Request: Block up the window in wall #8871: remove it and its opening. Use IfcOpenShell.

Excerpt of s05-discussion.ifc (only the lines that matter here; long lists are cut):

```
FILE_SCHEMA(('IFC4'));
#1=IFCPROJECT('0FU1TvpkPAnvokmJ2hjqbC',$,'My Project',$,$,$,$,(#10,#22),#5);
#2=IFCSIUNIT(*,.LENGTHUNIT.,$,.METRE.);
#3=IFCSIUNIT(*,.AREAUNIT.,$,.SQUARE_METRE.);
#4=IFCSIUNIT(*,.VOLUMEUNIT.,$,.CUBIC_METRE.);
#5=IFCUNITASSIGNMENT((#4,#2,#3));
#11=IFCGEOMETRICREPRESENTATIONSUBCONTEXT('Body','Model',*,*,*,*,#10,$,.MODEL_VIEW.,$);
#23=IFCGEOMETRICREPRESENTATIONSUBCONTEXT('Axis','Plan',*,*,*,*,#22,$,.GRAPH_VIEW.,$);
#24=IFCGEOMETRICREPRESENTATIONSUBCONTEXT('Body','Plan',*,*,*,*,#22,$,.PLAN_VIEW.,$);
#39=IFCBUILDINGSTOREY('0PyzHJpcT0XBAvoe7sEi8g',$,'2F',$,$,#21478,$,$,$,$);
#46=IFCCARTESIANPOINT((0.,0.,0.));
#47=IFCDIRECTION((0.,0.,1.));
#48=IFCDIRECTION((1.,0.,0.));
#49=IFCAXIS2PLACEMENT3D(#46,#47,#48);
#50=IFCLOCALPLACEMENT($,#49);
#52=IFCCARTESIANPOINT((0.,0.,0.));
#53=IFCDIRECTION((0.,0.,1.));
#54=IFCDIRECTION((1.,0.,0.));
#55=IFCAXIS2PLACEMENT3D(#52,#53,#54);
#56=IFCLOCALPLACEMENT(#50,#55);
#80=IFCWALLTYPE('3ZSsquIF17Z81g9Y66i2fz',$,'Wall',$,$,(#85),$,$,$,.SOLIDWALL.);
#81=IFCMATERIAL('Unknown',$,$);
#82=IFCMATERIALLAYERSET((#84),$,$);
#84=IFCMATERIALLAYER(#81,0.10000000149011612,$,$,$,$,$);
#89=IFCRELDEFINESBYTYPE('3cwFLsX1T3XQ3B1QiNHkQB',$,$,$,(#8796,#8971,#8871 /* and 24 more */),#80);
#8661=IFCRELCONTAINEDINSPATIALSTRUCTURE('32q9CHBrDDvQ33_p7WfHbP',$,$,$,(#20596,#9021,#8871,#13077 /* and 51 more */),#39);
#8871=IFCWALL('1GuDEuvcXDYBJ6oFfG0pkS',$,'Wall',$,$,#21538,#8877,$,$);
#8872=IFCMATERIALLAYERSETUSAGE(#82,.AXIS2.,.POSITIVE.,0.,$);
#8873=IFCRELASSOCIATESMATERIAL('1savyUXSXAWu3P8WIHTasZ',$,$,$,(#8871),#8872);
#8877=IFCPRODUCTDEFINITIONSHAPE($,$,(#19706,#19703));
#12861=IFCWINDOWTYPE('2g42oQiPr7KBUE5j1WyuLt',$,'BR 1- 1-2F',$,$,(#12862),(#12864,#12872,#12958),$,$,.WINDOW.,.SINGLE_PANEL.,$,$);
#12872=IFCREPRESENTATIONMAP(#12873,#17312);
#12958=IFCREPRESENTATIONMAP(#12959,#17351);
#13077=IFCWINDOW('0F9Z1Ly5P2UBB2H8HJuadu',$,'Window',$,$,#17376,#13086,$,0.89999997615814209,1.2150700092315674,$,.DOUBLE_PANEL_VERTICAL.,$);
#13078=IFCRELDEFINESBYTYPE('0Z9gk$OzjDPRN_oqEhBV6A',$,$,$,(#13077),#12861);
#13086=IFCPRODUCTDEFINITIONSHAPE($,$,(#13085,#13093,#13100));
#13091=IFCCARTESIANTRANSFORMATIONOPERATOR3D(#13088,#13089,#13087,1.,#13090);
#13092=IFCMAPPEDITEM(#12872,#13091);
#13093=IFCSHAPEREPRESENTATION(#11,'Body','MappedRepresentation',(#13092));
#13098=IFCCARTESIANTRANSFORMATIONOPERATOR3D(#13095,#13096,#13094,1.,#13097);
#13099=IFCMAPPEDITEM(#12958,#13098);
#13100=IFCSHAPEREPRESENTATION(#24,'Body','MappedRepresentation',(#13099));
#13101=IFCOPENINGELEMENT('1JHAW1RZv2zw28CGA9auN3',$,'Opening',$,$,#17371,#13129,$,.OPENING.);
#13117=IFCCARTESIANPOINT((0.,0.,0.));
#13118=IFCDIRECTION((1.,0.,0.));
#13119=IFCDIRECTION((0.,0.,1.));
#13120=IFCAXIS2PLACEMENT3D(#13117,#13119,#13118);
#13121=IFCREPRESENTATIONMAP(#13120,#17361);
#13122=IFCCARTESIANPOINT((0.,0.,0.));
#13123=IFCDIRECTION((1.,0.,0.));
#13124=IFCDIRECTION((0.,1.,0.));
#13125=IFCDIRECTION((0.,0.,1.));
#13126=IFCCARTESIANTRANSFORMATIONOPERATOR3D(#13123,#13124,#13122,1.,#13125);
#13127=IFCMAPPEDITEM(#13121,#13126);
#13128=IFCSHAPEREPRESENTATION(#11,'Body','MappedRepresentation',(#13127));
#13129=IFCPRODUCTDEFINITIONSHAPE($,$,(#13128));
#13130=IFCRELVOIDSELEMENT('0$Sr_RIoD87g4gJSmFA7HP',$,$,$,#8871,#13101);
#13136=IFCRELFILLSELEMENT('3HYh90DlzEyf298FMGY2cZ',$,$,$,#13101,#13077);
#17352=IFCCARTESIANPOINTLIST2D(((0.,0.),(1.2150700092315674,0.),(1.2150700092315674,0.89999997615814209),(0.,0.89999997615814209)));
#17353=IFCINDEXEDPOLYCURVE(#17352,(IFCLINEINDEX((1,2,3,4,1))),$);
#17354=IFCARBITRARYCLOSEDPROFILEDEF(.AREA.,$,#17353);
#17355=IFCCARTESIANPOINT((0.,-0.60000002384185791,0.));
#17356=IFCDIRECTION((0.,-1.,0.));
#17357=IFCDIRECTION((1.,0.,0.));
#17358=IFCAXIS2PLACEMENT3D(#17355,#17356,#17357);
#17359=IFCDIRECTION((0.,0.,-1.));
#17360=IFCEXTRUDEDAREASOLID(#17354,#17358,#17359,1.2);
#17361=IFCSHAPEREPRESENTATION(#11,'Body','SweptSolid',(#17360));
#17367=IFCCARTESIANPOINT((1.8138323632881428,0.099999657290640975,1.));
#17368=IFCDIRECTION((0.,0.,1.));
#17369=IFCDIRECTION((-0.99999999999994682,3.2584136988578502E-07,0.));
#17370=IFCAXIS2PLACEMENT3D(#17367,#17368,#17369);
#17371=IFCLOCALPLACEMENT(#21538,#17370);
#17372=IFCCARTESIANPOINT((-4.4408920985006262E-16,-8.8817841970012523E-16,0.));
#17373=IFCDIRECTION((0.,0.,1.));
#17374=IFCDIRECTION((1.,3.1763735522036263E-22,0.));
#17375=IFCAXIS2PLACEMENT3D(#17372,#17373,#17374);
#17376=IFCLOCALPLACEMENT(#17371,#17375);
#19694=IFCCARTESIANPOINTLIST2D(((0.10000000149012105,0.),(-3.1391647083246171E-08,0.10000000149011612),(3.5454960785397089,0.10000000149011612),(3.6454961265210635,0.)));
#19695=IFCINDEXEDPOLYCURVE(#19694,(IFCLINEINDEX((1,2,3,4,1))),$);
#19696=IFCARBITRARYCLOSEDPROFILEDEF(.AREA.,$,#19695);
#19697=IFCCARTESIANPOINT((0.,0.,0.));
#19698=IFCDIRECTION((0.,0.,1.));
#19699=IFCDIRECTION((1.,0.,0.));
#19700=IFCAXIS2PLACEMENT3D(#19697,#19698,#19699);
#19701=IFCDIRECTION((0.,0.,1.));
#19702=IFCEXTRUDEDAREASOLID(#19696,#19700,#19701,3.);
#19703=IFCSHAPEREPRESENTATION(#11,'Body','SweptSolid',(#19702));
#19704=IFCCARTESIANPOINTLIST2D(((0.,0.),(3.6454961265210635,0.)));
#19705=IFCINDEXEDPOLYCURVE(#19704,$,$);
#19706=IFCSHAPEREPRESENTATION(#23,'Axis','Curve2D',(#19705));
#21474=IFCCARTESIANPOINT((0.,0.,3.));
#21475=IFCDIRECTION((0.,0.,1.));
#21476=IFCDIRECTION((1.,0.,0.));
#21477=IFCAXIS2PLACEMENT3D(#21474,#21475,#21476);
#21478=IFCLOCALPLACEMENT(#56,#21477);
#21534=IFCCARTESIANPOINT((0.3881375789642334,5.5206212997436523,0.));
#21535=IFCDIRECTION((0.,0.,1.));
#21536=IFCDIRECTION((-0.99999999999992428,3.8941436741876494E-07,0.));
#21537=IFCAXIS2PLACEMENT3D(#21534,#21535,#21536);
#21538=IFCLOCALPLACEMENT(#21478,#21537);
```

```python
import ifcopenshell
import ifcopenshell.api.feature
import ifcopenshell.api.root
import ifcopenshell.geom
import ifcopenshell.util.shape

model = ifcopenshell.open("s05-discussion.ifc")
settings = ifcopenshell.geom.settings()


def volume(element):
    """Net volume in cubic metres, openings subtracted."""
    shape = ifcopenshell.geom.create_shape(settings, element)
    return ifcopenshell.util.shape.get_volume(shape.geometry)


window = model.by_id(13077)
opening = window.FillsVoids[0].RelatingOpeningElement
wall = opening.VoidsElements[0].RelatingBuildingElement
before = volume(wall)

ifcopenshell.api.root.remove_product(model, product=window)
ifcopenshell.api.feature.remove_feature(model, feature=opening)

after = volume(wall)

print(f"wall volume {before:.3f} -> {after:.3f} m3")

model.write("s05-discussion_rev.ifc")
```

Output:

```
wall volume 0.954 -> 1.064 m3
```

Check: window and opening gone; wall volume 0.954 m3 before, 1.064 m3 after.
